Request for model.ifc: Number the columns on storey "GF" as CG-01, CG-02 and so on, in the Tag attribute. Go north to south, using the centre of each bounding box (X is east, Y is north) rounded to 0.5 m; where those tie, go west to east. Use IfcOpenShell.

First a look at what the model holds.

```python
import ifcopenshell
import ifcopenshell.util.element
import ifcopenshell.util.placement

model = ifcopenshell.open("model.ifc")
print(model.schema)
storey = next(s for s in model.by_type("IfcBuildingStorey") if s.Name == "GF")
columns = [e for e in ifcopenshell.util.element.get_decomposition(storey) if e.is_a("IfcColumn")]
for e in sorted(columns, key=lambda e: e.id()):
    origin = ifcopenshell.util.placement.get_local_placement(e.ObjectPlacement)[:3, 3]
    print(e.id(), e.Tag, e.Name, origin.round(2) + 0.0, sep=" | ")
```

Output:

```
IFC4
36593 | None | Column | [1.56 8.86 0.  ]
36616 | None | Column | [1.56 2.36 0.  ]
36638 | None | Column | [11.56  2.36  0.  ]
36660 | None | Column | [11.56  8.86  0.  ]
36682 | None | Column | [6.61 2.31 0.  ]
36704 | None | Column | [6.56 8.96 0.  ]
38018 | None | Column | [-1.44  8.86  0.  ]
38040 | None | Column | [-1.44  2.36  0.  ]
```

```python
import ifcopenshell
import ifcopenshell.geom
import ifcopenshell.util.element
import ifcopenshell.util.shape

model = ifcopenshell.open("model.ifc")
settings = ifcopenshell.geom.settings()
settings.set("use-world-coords", True)


def centre(element):
    shape = ifcopenshell.geom.create_shape(settings, element)
    return ifcopenshell.util.shape.get_bbox_centroid(shape.geometry)


storey = next(s for s in model.by_type("IfcBuildingStorey") if s.Name == "GF")
columns = [e for e in ifcopenshell.util.element.get_decomposition(storey) if e.is_a("IfcColumn")]

# Insertion points can sit at a corner or the storey origin, so sort by the geometry (in metres).
centres = {e: centre(e) for e in columns}
columns.sort(key=lambda e: (-round(centres[e][1] / 0.5), centres[e][0]))

for i, e in enumerate(columns, start=1):
    number = f"CG-{i:02d}"
    e.Tag = number
    print(e.id(), number)

model.write("model_v2.ifc")
```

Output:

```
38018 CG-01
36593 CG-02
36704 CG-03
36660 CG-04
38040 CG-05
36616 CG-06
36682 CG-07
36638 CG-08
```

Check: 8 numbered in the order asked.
